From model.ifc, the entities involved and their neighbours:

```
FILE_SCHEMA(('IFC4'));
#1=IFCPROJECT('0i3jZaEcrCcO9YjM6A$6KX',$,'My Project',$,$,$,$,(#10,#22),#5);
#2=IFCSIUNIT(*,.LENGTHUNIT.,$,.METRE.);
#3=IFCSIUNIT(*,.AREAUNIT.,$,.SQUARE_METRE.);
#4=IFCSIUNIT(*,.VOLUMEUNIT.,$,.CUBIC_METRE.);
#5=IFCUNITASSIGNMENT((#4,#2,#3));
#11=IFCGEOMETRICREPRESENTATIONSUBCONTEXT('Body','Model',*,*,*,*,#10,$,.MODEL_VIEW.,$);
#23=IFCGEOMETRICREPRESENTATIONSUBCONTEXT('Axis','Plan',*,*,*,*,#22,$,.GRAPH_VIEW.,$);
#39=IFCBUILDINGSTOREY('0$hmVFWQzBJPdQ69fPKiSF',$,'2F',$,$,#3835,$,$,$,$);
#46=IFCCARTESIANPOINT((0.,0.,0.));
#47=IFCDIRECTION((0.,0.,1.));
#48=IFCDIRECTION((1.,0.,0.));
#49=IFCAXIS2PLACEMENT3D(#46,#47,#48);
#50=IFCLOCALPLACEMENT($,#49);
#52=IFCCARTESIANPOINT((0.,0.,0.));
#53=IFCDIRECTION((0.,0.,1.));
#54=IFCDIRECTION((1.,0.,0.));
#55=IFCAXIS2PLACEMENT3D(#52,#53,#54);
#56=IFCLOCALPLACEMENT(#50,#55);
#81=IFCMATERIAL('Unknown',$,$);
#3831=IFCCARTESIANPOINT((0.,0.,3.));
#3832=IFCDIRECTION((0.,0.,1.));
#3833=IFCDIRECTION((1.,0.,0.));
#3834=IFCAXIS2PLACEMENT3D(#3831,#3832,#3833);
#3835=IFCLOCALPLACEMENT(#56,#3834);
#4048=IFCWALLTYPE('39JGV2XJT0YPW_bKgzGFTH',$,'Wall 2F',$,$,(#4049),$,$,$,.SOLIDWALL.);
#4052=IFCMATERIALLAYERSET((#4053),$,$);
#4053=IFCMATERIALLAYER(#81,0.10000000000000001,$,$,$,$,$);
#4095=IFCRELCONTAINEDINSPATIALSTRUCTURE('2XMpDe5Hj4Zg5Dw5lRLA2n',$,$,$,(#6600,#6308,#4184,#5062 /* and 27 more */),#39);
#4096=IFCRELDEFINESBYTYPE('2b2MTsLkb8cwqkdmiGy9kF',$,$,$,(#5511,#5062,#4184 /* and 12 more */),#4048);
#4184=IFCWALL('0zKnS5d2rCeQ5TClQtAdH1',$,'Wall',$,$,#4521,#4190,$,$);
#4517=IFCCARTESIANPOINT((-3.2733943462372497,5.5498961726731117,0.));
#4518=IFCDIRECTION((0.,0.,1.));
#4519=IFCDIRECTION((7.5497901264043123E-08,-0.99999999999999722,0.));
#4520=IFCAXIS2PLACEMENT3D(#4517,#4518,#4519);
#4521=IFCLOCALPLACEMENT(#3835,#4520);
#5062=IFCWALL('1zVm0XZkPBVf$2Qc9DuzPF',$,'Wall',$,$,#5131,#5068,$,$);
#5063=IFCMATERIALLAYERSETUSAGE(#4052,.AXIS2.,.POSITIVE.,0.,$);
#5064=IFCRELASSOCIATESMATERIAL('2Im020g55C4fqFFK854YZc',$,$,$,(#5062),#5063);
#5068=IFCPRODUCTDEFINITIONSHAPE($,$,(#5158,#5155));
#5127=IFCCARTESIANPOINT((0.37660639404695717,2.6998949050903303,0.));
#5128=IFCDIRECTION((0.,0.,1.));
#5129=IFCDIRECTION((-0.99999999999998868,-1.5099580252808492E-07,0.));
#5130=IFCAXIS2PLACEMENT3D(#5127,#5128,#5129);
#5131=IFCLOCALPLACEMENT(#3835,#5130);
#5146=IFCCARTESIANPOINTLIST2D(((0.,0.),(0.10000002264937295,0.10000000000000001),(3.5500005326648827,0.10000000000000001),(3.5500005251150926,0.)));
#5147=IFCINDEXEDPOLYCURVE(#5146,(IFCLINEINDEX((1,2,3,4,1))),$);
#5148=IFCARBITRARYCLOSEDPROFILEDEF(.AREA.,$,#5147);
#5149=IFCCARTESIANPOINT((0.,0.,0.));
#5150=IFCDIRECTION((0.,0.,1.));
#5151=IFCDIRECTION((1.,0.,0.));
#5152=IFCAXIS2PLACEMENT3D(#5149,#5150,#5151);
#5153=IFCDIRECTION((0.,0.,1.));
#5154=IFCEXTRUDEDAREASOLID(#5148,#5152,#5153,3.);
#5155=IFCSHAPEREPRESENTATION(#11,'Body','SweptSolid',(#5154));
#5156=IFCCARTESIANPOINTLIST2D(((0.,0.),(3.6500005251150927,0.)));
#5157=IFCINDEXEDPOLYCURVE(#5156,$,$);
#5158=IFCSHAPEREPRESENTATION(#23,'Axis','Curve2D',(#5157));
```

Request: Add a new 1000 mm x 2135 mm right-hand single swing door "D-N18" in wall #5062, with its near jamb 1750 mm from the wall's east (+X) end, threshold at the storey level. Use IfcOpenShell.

```python
import numpy as np
import ifcopenshell
import ifcopenshell.api.feature
import ifcopenshell.api.geometry
import ifcopenshell.api.root
import ifcopenshell.api.spatial
import ifcopenshell.geom
import ifcopenshell.util.element
import ifcopenshell.util.placement
import ifcopenshell.util.representation
import ifcopenshell.util.shape
import ifcopenshell.util.unit

model = ifcopenshell.open("model.ifc")
unit_scale = ifcopenshell.util.unit.calculate_unit_scale(model)
settings = ifcopenshell.geom.settings()


def volume(element):
    """Net volume in cubic metres, openings subtracted."""
    shape = ifcopenshell.geom.create_shape(settings, element)
    return ifcopenshell.util.shape.get_volume(shape.geometry)


wall = model.by_id(5062)
storey = ifcopenshell.util.element.get_container(wall, ifc_class="IfcBuildingStorey")
context = ifcopenshell.util.representation.get_context(model, "Model", "Body", "MODEL_VIEW")
before = volume(wall)

width, height, from_end, sill = 1, 2.135, 1.75, 0.0  # metres

# The wall runs along its own X axis, and the end named is its -X end.
wall_shape = ifcopenshell.geom.create_shape(settings, wall)
x, y, z = ifcopenshell.util.shape.get_vertices(wall_shape.geometry).T
start = x.min() + from_end
face, thickness = float(y.min()), float(y.max() - y.min())
wall_matrix = ifcopenshell.util.placement.get_local_placement(wall.ObjectPlacement)
level = ifcopenshell.util.placement.get_local_placement(storey.ObjectPlacement)[2, 3]


def in_wall(x, y):
    """Placement at x, y metres in the wall's axes, at sill height."""
    matrix = wall_matrix.copy()
    matrix[:, 3] = wall_matrix @ np.array([x / unit_scale, y / unit_scale, 0.0, 1.0])
    matrix[2, 3] = level + sill / unit_scale
    return matrix


# Opening: a box that overshoots both wall faces by 50 mm.
opening = ifcopenshell.api.root.create_entity(model, ifc_class="IfcOpeningElement", predefined_type="OPENING")
box = ifcopenshell.api.geometry.add_wall_representation(
    model, context=context, length=width, height=height, thickness=thickness + 0.1
)
ifcopenshell.api.geometry.assign_representation(model, product=opening, representation=box)
ifcopenshell.api.geometry.edit_object_placement(model, product=opening, matrix=in_wall(start, face - 0.05), is_si=False)
ifcopenshell.api.feature.add_feature(model, feature=opening, element=wall)

door = ifcopenshell.api.root.create_entity(model, ifc_class="IfcDoor", name="D-N18", predefined_type="DOOR")
door.OverallWidth, door.OverallHeight = width / unit_scale, height / unit_scale
door.OperationType = "SINGLE_SWING_RIGHT"
body = ifcopenshell.api.geometry.add_door_representation(
    model,
    context=context,
    overall_width=door.OverallWidth,
    overall_height=door.OverallHeight,
    operation_type="SINGLE_SWING_RIGHT",
    lining_properties={"LiningDepth": thickness / unit_scale, "ThresholdDepth": thickness / unit_scale},
)
ifcopenshell.api.geometry.assign_representation(model, product=door, representation=body)
ifcopenshell.api.spatial.assign_container(model, products=[door], relating_structure=storey)
ifcopenshell.api.feature.add_filling(model, opening=opening, element=door)

# The lining spans the wall, so the door starts at the wall face.
ifcopenshell.api.geometry.edit_object_placement(model, product=door, matrix=in_wall(start, face), is_si=False)

after = volume(wall)

print(f"wall volume {before:.3f} -> {after:.3f} m3")

model.write("model_v2.ifc")
```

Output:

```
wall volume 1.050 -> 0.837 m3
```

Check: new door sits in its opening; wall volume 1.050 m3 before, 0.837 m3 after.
